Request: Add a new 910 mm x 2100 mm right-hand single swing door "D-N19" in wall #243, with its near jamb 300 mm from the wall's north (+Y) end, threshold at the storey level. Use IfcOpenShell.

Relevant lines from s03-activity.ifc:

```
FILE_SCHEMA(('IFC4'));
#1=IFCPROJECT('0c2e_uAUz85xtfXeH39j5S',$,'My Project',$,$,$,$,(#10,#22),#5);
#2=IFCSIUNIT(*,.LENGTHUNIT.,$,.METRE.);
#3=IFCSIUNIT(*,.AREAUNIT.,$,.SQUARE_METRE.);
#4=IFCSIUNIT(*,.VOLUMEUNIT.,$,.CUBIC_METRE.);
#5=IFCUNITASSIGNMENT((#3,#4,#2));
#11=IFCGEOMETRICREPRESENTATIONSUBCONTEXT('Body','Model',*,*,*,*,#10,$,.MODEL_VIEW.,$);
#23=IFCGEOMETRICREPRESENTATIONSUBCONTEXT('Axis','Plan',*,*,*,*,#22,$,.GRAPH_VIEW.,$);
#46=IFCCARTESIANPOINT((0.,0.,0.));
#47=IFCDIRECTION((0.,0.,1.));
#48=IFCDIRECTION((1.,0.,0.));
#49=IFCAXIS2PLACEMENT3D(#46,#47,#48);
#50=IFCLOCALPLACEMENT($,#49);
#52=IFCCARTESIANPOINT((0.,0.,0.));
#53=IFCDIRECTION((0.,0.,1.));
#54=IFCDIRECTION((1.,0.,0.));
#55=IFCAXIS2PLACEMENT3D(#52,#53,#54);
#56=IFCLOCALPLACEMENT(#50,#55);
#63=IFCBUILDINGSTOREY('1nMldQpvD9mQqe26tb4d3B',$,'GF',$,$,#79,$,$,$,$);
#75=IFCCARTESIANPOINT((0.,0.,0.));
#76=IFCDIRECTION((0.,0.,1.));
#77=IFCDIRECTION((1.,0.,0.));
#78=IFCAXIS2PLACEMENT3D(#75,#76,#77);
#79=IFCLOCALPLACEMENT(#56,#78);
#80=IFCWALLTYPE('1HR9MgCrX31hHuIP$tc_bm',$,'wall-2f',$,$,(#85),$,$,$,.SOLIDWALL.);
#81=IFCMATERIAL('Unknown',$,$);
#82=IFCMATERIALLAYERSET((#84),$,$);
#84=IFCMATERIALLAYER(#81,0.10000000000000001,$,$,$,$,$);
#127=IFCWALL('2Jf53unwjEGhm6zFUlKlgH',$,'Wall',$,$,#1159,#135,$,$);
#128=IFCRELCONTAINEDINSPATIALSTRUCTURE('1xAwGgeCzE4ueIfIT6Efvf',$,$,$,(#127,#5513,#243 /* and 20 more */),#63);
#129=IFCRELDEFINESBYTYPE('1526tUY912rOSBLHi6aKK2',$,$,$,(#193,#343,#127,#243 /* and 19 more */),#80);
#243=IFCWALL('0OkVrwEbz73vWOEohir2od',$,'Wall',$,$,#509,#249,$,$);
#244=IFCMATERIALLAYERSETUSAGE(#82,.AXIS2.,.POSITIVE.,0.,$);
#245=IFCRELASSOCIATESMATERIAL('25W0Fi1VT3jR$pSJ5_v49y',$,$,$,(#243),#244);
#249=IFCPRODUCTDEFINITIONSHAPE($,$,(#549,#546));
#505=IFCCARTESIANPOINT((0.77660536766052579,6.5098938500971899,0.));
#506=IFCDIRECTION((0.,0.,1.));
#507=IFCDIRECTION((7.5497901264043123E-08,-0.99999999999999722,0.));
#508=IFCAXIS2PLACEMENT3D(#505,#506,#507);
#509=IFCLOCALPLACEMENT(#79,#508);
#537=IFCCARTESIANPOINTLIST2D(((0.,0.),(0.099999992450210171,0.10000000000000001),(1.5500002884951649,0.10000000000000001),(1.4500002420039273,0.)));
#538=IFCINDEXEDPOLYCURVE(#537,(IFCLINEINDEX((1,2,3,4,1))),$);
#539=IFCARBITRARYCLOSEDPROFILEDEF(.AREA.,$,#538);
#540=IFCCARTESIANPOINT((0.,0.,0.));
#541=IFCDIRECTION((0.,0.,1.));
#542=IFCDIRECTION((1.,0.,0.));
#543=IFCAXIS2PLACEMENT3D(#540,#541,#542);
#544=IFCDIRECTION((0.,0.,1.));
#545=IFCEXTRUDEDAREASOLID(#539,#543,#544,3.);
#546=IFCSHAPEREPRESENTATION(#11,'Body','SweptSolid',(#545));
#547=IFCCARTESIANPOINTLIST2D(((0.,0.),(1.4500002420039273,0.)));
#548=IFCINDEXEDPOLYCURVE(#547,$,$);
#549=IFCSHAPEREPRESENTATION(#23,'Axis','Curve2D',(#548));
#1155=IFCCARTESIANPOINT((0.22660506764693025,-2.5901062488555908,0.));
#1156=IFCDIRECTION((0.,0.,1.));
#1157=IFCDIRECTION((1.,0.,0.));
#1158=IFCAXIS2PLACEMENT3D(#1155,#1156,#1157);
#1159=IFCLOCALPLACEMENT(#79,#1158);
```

```python
import numpy as np
import ifcopenshell
import ifcopenshell.api.feature
import ifcopenshell.api.geometry
import ifcopenshell.api.root
import ifcopenshell.api.spatial
import ifcopenshell.geom
import ifcopenshell.util.element
import ifcopenshell.util.placement
import ifcopenshell.util.representation
import ifcopenshell.util.shape
import ifcopenshell.util.unit

model = ifcopenshell.open("s03-activity.ifc")
unit_scale = ifcopenshell.util.unit.calculate_unit_scale(model)
settings = ifcopenshell.geom.settings()


def volume(element):
    """Net volume in cubic metres, openings subtracted."""
    shape = ifcopenshell.geom.create_shape(settings, element)
    return ifcopenshell.util.shape.get_volume(shape.geometry)


wall = model.by_guid("0OkVrwEbz73vWOEohir2od")
storey = ifcopenshell.util.element.get_container(wall, ifc_class="IfcBuildingStorey")
context = ifcopenshell.util.representation.get_context(model, "Model", "Body", "MODEL_VIEW")
before = volume(wall)

width, height, from_end, sill = 0.91, 2.1, 0.3, 0.0  # metres

# The wall runs along its own X axis, and the end named is its -X end.
wall_shape = ifcopenshell.geom.create_shape(settings, wall)
x, y, z = ifcopenshell.util.shape.get_vertices(wall_shape.geometry).T
start = x.min() + from_end
face, thickness = float(y.min()), float(y.max() - y.min())
wall_matrix = ifcopenshell.util.placement.get_local_placement(wall.ObjectPlacement)
level = ifcopenshell.util.placement.get_local_placement(storey.ObjectPlacement)[2, 3]


def in_wall(x, y):
    """Placement at x, y metres in the wall's axes, at sill height."""
    matrix = wall_matrix.copy()
    matrix[:, 3] = wall_matrix @ np.array([x / unit_scale, y / unit_scale, 0.0, 1.0])
    matrix[2, 3] = level + sill / unit_scale
    return matrix


# Opening: a box that overshoots both wall faces by 50 mm.
opening = ifcopenshell.api.root.create_entity(model, ifc_class="IfcOpeningElement", predefined_type="OPENING")
box = ifcopenshell.api.geometry.add_wall_representation(
    model, context=context, length=width, height=height, thickness=thickness + 0.1
)
ifcopenshell.api.geometry.assign_representation(model, product=opening, representation=box)
ifcopenshell.api.geometry.edit_object_placement(model, product=opening, matrix=in_wall(start, face - 0.05), is_si=False)
ifcopenshell.api.feature.add_feature(model, feature=opening, element=wall)

door = ifcopenshell.api.root.create_entity(model, ifc_class="IfcDoor", name="D-N19", predefined_type="DOOR")
door.OverallWidth, door.OverallHeight = width / unit_scale, height / unit_scale
door.OperationType = "SINGLE_SWING_RIGHT"
body = ifcopenshell.api.geometry.add_door_representation(
    model,
    context=context,
    overall_width=door.OverallWidth,
    overall_height=door.OverallHeight,
    operation_type="SINGLE_SWING_RIGHT",
    lining_properties={"LiningDepth": thickness / unit_scale, "ThresholdDepth": thickness / unit_scale},
)
ifcopenshell.api.geometry.assign_representation(model, product=door, representation=body)
ifcopenshell.api.spatial.assign_container(model, products=[door], relating_structure=storey)
ifcopenshell.api.feature.add_filling(model, opening=opening, element=door)

# The lining spans the wall, so the door starts at the wall face.
ifcopenshell.api.geometry.edit_object_placement(model, product=door, matrix=in_wall(start, face), is_si=False)

after = volume(wall)

print(f"wall volume {before:.3f} -> {after:.3f} m3")

model.write("s03-activity_v2.ifc")
```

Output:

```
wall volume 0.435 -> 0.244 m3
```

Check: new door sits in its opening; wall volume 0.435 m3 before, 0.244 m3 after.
